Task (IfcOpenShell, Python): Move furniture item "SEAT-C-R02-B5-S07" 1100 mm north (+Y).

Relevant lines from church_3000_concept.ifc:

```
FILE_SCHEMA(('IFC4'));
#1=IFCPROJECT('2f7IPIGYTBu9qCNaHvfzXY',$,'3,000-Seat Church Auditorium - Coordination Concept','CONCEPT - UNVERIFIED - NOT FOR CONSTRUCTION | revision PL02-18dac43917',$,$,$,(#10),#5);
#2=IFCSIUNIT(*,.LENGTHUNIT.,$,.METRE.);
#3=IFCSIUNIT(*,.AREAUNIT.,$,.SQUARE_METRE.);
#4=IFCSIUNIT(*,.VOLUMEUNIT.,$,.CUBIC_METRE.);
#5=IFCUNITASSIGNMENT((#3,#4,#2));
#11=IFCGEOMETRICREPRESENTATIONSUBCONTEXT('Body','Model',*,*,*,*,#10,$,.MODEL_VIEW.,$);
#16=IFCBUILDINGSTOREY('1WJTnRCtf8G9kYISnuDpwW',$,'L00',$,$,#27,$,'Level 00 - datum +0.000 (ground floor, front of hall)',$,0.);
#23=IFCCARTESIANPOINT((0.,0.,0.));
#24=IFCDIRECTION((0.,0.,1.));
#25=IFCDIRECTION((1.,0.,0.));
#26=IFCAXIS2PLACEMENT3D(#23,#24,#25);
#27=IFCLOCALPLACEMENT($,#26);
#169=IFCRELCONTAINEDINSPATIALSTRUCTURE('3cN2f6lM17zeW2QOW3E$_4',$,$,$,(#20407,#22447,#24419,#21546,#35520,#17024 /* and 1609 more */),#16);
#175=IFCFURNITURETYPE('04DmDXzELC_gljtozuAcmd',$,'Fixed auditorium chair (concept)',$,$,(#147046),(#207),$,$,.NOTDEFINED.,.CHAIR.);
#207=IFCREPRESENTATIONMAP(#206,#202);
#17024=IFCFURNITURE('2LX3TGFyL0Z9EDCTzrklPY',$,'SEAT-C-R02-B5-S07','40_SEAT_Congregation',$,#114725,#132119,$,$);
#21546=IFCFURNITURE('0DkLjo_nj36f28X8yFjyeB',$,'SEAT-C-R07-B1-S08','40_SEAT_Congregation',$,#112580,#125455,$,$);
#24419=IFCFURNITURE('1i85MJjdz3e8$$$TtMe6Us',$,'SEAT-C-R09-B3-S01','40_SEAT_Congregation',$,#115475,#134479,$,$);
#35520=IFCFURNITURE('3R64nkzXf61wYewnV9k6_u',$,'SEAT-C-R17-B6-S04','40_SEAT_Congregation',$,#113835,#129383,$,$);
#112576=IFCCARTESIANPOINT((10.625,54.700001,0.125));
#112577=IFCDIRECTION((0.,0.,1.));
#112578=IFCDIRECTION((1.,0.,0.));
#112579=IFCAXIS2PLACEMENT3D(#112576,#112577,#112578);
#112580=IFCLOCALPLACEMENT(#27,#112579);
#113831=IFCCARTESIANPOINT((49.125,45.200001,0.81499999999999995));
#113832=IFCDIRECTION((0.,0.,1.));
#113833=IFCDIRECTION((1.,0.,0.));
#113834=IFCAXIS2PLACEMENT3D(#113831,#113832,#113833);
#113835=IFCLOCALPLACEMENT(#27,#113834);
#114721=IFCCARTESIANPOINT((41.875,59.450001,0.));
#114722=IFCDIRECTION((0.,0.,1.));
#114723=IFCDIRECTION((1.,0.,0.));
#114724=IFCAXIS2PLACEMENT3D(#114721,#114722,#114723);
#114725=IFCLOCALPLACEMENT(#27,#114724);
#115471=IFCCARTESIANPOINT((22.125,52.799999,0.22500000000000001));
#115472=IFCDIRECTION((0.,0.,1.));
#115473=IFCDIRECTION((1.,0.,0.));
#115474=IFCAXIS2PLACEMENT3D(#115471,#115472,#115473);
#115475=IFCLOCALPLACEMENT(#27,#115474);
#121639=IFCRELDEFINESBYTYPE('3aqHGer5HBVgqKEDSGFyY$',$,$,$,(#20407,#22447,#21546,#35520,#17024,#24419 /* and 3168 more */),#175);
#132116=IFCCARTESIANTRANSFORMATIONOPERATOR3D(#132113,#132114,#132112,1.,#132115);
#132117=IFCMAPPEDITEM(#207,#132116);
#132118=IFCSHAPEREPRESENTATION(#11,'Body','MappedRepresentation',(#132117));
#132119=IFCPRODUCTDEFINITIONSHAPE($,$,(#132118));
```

```python
import ifcopenshell
import ifcopenshell.api.geometry
import ifcopenshell.util.placement

model = ifcopenshell.open("church_3000_concept.ifc")

item = model.by_guid("2LX3TGFyL0Z9EDCTzrklPY")
matrix = ifcopenshell.util.placement.get_local_placement(item.ObjectPlacement)
matrix[1, 3] += 1.1
ifcopenshell.api.geometry.edit_object_placement(model, product=item, matrix=matrix, is_si=False)

print(ifcopenshell.util.placement.get_local_placement(item.ObjectPlacement).round(3) + 0.0)

model.write("church_3000_concept_edited.ifc")
```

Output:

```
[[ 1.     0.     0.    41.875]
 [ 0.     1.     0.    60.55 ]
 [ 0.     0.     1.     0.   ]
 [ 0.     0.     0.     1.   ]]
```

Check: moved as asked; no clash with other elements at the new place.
